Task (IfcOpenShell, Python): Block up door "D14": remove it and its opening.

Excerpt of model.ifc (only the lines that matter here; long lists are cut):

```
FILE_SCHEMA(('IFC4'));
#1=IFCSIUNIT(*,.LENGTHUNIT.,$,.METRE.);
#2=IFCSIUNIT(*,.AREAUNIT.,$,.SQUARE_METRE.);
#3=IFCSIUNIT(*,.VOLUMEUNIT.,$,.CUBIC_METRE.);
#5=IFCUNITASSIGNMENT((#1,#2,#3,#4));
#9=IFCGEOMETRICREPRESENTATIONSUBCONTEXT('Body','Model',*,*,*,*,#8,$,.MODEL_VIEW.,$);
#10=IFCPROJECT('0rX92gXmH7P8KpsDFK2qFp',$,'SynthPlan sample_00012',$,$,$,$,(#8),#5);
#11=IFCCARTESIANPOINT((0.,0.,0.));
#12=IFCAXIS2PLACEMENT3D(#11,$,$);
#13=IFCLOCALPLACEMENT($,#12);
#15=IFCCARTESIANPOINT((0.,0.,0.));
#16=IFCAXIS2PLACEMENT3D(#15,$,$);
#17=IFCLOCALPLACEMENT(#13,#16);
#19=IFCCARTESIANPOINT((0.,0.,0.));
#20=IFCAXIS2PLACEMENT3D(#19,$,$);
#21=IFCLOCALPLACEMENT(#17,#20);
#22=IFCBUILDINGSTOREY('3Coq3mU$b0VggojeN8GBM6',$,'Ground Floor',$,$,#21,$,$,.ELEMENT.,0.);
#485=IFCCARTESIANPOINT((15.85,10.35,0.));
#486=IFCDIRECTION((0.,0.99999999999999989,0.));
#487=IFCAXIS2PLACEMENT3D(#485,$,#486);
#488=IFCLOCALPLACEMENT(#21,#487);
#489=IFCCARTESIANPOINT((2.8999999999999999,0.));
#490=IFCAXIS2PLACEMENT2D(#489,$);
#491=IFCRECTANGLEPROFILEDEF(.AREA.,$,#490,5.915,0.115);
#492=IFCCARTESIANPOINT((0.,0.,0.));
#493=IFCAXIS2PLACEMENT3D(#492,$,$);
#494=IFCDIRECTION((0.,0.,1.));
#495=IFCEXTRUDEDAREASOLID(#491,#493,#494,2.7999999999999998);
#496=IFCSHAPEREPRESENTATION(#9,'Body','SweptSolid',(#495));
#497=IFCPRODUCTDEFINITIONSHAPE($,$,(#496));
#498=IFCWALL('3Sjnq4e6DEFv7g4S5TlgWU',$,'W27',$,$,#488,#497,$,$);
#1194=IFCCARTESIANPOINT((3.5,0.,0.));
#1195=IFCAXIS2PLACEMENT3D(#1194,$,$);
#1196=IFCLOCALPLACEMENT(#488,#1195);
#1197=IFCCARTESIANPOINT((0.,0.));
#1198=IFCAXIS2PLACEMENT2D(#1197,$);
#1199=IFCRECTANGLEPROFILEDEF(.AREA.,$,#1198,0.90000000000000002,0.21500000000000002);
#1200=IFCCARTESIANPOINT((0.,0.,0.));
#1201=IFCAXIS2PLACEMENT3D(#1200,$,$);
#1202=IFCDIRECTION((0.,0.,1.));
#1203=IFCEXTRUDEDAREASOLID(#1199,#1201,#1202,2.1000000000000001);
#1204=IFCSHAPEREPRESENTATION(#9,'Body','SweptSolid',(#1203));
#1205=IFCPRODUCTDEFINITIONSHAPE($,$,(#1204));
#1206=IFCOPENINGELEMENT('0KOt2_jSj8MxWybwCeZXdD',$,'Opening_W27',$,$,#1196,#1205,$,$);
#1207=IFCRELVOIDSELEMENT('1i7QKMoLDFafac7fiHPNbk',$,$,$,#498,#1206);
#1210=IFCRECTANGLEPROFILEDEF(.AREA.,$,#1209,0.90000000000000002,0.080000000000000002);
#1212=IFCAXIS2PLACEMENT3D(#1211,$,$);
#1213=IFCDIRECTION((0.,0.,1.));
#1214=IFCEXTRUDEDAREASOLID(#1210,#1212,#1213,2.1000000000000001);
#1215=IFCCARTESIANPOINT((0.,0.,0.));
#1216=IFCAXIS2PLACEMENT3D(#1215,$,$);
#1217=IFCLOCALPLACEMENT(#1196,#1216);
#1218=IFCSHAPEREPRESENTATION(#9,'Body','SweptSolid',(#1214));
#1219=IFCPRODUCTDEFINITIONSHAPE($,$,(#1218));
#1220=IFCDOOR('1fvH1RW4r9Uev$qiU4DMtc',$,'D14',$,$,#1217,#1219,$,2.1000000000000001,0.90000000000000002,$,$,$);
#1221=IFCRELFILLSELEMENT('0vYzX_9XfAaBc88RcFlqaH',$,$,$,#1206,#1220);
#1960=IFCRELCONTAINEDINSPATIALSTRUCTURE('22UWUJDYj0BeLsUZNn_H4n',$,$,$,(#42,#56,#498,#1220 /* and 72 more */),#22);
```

```python
import ifcopenshell
import ifcopenshell.api.feature
import ifcopenshell.api.root
import ifcopenshell.geom
import ifcopenshell.util.shape

model = ifcopenshell.open("model.ifc")
settings = ifcopenshell.geom.settings()


def volume(element):
    """Net volume in cubic metres, openings subtracted."""
    shape = ifcopenshell.geom.create_shape(settings, element)
    return ifcopenshell.util.shape.get_volume(shape.geometry)


door = model.by_guid("1fvH1RW4r9Uev$qiU4DMtc")
opening = door.FillsVoids[0].RelatingOpeningElement
wall = opening.VoidsElements[0].RelatingBuildingElement
before = volume(wall)

ifcopenshell.api.root.remove_product(model, product=door)
ifcopenshell.api.feature.remove_feature(model, feature=opening)

after = volume(wall)

print(f"wall volume {before:.3f} -> {after:.3f} m3")

model.write("model-out.ifc")
```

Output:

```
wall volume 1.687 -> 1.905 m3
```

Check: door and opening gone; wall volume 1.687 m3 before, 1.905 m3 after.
